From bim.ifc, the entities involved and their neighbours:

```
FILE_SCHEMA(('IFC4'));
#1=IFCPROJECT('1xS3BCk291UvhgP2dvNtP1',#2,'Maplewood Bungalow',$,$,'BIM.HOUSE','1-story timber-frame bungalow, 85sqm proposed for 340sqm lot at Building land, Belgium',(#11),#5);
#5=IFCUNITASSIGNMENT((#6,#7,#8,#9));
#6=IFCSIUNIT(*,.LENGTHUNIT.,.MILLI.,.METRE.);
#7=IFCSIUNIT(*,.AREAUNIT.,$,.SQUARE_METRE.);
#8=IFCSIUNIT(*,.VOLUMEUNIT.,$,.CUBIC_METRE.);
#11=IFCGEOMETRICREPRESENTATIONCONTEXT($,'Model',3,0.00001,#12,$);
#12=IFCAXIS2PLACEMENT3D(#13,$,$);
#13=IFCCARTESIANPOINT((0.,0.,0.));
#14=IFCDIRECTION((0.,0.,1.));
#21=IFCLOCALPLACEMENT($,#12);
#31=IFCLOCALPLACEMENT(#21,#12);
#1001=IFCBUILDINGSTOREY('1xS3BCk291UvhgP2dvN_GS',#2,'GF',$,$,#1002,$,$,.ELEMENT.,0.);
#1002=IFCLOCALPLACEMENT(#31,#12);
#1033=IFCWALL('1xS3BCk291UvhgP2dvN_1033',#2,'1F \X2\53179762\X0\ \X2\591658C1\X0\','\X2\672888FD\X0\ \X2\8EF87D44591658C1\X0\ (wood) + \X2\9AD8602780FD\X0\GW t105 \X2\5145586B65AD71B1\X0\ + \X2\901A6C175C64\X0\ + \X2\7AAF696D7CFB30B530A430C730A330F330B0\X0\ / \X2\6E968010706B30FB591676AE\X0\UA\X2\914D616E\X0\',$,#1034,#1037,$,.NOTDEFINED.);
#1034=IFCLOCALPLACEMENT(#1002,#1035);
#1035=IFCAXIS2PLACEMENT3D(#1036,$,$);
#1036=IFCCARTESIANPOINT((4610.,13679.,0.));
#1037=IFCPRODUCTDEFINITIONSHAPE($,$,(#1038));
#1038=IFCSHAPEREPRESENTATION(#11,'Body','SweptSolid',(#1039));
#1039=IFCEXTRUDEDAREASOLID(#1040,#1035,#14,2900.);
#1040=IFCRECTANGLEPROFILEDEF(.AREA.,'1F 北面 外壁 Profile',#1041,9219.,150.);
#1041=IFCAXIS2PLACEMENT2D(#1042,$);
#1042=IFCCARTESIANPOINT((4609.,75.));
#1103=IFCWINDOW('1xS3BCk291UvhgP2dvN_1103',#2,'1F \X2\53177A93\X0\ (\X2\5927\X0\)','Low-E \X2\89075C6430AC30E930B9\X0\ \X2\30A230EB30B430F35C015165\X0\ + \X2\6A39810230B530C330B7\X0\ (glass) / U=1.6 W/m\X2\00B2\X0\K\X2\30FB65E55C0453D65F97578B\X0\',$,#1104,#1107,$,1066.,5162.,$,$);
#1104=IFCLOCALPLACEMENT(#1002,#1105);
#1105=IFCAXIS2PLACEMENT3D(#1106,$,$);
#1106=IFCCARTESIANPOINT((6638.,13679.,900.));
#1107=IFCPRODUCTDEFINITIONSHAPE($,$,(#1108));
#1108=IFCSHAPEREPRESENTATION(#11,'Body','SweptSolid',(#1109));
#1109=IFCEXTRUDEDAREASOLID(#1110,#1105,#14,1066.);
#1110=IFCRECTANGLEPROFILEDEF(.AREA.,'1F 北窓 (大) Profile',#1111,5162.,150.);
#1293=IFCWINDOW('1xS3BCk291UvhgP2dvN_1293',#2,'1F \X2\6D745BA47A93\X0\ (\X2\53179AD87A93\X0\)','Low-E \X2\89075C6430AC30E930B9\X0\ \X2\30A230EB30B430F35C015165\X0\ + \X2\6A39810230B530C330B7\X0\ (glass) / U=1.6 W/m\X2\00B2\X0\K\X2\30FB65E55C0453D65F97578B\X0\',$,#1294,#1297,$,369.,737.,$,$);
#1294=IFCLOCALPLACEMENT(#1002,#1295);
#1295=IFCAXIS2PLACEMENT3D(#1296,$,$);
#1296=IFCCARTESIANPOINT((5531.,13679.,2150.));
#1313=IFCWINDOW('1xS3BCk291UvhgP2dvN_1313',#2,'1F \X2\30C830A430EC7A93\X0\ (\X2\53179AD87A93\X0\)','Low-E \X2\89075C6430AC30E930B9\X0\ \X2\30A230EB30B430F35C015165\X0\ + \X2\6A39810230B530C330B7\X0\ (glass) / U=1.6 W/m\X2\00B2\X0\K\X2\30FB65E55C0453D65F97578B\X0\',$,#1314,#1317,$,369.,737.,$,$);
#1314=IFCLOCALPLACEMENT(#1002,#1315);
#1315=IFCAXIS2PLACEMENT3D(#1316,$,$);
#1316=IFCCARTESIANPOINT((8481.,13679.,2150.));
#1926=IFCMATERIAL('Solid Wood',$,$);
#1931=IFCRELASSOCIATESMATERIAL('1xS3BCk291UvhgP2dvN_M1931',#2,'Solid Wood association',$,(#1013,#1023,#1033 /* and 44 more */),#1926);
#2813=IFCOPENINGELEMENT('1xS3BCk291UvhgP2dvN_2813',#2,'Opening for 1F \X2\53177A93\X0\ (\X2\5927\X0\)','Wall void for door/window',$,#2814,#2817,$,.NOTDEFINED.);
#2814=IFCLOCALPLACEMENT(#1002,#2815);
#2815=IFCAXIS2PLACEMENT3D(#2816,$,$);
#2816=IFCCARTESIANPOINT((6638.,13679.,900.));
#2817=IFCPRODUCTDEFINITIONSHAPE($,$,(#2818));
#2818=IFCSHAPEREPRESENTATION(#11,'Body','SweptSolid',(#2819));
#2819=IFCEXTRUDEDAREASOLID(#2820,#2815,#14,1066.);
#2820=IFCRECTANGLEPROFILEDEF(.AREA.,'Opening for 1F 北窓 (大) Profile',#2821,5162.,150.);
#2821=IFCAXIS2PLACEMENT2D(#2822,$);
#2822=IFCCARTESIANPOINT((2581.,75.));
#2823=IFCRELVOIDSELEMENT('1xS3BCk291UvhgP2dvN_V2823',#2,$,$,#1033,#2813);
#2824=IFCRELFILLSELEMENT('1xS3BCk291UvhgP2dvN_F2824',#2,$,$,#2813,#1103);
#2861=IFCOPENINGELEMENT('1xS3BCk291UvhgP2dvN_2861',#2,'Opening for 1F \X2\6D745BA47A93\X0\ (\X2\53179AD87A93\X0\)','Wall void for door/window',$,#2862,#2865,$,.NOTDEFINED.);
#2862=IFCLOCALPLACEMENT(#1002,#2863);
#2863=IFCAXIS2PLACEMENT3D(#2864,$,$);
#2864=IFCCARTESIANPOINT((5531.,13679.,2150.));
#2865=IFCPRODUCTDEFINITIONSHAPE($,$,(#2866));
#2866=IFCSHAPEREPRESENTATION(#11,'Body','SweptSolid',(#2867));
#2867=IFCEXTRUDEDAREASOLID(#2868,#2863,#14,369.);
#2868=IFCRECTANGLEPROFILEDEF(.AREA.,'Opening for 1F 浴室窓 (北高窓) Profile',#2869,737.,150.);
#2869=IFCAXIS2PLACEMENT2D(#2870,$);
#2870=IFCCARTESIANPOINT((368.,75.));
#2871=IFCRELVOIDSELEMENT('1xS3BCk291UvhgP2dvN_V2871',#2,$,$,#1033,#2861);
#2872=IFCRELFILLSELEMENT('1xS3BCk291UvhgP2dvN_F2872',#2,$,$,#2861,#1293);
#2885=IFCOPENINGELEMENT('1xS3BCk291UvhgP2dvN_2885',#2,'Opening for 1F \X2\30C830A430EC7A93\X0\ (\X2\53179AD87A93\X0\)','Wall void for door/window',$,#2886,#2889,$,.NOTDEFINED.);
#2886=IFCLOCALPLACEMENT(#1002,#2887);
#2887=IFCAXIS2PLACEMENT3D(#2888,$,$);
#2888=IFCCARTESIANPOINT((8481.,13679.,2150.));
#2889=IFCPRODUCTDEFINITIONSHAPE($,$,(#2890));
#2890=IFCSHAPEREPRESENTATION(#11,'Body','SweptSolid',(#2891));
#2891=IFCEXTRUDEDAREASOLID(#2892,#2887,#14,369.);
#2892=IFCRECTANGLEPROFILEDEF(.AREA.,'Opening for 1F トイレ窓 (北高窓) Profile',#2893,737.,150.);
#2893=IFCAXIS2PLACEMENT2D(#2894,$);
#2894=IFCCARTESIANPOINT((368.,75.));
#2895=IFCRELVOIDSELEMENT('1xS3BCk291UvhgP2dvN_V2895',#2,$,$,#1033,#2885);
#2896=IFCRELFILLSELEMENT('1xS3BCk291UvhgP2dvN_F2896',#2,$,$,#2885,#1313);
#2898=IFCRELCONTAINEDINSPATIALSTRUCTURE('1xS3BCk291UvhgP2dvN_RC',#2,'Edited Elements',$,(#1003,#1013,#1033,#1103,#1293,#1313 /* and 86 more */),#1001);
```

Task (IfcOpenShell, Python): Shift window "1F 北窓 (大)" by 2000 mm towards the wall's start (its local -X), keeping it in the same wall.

```python
import ifcopenshell
import ifcopenshell.api.geometry
import ifcopenshell.util.placement

model = ifcopenshell.open("bim.ifc")

window = model.by_guid("1xS3BCk291UvhgP2dvN_1103")
opening = window.FillsVoids[0].RelatingOpeningElement
wall = opening.VoidsElements[0].RelatingBuildingElement

wall_matrix = ifcopenshell.util.placement.get_local_placement(wall.ObjectPlacement)
shift = wall_matrix[:3, 0] * -2000.0
before = ifcopenshell.util.placement.get_local_placement(window.ObjectPlacement)[:3, 3].copy()

# The window is not placed relative to its opening, so move both.
for product in (opening, window):
    matrix = ifcopenshell.util.placement.get_local_placement(product.ObjectPlacement)
    matrix[:3, 3] += shift
    ifcopenshell.api.geometry.edit_object_placement(model, product=product, matrix=matrix, is_si=False)

after = ifcopenshell.util.placement.get_local_placement(window.ObjectPlacement)[:3, 3]
print("window moved by", (after - before).round(3) + 0.0)

model.write("bim_updated.ifc")
```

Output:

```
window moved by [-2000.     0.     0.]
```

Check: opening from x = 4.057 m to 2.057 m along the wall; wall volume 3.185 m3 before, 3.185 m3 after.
